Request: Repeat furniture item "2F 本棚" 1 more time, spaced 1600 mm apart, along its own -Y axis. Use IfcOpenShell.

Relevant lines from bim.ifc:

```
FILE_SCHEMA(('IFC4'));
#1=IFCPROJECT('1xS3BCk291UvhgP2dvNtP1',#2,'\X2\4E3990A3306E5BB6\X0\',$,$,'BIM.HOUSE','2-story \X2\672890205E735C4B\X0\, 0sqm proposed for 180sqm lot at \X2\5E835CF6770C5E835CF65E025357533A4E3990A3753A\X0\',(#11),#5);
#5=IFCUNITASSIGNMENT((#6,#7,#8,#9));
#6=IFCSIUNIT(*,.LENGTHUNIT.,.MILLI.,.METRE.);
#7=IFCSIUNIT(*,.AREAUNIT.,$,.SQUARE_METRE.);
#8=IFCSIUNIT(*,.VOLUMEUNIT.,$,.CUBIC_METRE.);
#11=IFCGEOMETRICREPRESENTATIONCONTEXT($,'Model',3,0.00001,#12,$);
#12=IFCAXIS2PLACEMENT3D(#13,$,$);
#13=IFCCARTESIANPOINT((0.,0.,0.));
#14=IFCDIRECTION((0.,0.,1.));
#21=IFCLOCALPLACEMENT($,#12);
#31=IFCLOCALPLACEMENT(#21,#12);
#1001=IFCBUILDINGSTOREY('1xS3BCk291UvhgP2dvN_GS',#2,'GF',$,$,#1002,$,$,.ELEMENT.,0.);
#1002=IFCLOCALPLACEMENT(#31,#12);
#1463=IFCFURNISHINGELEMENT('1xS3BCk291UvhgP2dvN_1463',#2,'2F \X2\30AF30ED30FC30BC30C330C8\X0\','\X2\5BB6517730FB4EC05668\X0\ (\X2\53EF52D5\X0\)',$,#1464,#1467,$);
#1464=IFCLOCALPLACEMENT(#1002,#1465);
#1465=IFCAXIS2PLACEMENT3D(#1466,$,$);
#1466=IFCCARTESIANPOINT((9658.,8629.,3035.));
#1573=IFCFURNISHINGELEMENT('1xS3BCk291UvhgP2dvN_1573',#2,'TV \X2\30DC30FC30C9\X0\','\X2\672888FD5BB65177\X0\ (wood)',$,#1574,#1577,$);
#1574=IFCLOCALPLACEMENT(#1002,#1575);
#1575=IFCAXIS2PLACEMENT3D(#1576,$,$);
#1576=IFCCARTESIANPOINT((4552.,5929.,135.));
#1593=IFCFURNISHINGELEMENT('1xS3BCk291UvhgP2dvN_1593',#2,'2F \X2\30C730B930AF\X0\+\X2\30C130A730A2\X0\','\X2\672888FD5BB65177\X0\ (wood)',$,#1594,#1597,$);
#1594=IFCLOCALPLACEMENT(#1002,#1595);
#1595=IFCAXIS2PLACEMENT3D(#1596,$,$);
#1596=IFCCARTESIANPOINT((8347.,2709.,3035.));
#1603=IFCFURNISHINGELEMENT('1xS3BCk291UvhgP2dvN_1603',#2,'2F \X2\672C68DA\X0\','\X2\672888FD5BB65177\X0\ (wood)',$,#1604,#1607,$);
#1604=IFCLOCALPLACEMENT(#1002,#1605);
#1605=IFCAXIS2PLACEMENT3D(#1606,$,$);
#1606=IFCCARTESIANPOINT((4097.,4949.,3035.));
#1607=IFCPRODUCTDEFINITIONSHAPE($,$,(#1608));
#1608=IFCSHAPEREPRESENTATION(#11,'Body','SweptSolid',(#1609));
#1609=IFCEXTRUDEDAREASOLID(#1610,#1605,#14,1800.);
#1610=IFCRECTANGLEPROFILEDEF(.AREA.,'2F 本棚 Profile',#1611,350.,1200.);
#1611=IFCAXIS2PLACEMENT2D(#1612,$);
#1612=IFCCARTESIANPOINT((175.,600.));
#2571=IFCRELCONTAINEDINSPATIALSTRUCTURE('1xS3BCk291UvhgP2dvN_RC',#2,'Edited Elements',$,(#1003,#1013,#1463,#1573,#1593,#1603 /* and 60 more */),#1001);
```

```python
import ifcopenshell
import ifcopenshell.api.geometry
import ifcopenshell.api.root
import ifcopenshell.util.element
import ifcopenshell.util.placement

model = ifcopenshell.open("bim.ifc")


def reuse_history(source, copy):
    """copy_class also copies each property set's owner history, people and application; keep the originals."""
    for rel in copy.IsDefinedBy:
        if rel.is_a("IfcRelDefinesByProperties") and (history := rel.RelatingPropertyDefinition.OwnerHistory):
            rel.RelatingPropertyDefinition.OwnerHistory = source.OwnerHistory
            ifcopenshell.util.element.remove_deep2(model, history)


source = model.by_guid("1xS3BCk291UvhgP2dvN_1603")
base = ifcopenshell.util.placement.get_local_placement(source.ObjectPlacement)
step = -base[:3, 1] * 1600.0

for i in range(1, 2):
    copy = ifcopenshell.api.root.copy_class(model, product=source)
    copy.Representation = ifcopenshell.util.element.copy_deep(
        model, source.Representation, exclude=["IfcGeometricRepresentationContext", "IfcRepresentationMap"]
    )
    reuse_history(source, copy)
    matrix = base.copy()
    matrix[:3, 3] += i * step
    print("added at", matrix[:3, 3].round(3) + 0.0)
    ifcopenshell.api.geometry.edit_object_placement(model, product=copy, matrix=matrix, is_si=False)

model.write("bim_edited.ifc")
```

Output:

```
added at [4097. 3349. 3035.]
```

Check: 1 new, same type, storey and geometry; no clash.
